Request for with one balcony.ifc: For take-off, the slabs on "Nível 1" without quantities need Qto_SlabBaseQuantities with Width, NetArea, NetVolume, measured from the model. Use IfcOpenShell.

First a look at what the model holds.

```python
import ifcopenshell
import ifcopenshell.util.element
import ifcopenshell.util.unit

model = ifcopenshell.open("with one balcony.ifc")
print(model.schema)
for unit_type in ("LENGTHUNIT", "AREAUNIT", "VOLUMEUNIT"):
    print(unit_type, ifcopenshell.util.unit.calculate_unit_scale(model, unit_type))
storey = next(s for s in model.by_type("IfcBuildingStorey") if s.Name == "Nível 1")
slabs = [e for e in ifcopenshell.util.element.get_decomposition(storey) if e.is_a("IfcSlab")]
for e in sorted(slabs, key=lambda e: e.id()):
    print(e.id(), e.is_a(), e.Name, list(ifcopenshell.util.element.get_psets(e, qtos_only=True)), sep=" | ")
```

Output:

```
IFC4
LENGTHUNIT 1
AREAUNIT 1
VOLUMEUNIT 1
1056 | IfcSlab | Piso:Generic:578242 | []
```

```python
import ifcopenshell
import ifcopenshell.api.pset
import ifcopenshell.geom
import ifcopenshell.util.element
import ifcopenshell.util.shape
import ifcopenshell.util.unit

model = ifcopenshell.open("with one balcony.ifc")
unit_scale = ifcopenshell.util.unit.calculate_unit_scale(model)
area_scale = ifcopenshell.util.unit.calculate_unit_scale(model, "AREAUNIT")
volume_scale = ifcopenshell.util.unit.calculate_unit_scale(model, "VOLUMEUNIT")
settings = ifcopenshell.geom.settings()

storey = next(s for s in model.by_type("IfcBuildingStorey") if s.Name == "Nível 1")
slabs = [e for e in ifcopenshell.util.element.get_decomposition(storey) if e.is_a("IfcSlab")]

for e in sorted(slabs, key=lambda e: e.id()):
    if ifcopenshell.util.element.get_psets(e, qtos_only=True, should_inherit=False):
        continue
    # Geometry comes back in metres, in the element's own axes.
    shape = ifcopenshell.geom.create_shape(settings, e)
    values = {
        "Width": ifcopenshell.util.shape.get_z(shape.geometry) / unit_scale,
        "NetArea": ifcopenshell.util.shape.get_footprint_area(shape.geometry) / area_scale,
        "NetVolume": ifcopenshell.util.shape.get_volume(shape.geometry) / volume_scale,
    }
    qto = ifcopenshell.api.pset.add_qto(model, product=e, name="Qto_SlabBaseQuantities")
    ifcopenshell.api.pset.edit_qto(model, qto=qto, properties=values)
    print(e.id(), {k: round(v, 3) for k, v in values.items()})

model.write("with one balcony_updated.ifc")
```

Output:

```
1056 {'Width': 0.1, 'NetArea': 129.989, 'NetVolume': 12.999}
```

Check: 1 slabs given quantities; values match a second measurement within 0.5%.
